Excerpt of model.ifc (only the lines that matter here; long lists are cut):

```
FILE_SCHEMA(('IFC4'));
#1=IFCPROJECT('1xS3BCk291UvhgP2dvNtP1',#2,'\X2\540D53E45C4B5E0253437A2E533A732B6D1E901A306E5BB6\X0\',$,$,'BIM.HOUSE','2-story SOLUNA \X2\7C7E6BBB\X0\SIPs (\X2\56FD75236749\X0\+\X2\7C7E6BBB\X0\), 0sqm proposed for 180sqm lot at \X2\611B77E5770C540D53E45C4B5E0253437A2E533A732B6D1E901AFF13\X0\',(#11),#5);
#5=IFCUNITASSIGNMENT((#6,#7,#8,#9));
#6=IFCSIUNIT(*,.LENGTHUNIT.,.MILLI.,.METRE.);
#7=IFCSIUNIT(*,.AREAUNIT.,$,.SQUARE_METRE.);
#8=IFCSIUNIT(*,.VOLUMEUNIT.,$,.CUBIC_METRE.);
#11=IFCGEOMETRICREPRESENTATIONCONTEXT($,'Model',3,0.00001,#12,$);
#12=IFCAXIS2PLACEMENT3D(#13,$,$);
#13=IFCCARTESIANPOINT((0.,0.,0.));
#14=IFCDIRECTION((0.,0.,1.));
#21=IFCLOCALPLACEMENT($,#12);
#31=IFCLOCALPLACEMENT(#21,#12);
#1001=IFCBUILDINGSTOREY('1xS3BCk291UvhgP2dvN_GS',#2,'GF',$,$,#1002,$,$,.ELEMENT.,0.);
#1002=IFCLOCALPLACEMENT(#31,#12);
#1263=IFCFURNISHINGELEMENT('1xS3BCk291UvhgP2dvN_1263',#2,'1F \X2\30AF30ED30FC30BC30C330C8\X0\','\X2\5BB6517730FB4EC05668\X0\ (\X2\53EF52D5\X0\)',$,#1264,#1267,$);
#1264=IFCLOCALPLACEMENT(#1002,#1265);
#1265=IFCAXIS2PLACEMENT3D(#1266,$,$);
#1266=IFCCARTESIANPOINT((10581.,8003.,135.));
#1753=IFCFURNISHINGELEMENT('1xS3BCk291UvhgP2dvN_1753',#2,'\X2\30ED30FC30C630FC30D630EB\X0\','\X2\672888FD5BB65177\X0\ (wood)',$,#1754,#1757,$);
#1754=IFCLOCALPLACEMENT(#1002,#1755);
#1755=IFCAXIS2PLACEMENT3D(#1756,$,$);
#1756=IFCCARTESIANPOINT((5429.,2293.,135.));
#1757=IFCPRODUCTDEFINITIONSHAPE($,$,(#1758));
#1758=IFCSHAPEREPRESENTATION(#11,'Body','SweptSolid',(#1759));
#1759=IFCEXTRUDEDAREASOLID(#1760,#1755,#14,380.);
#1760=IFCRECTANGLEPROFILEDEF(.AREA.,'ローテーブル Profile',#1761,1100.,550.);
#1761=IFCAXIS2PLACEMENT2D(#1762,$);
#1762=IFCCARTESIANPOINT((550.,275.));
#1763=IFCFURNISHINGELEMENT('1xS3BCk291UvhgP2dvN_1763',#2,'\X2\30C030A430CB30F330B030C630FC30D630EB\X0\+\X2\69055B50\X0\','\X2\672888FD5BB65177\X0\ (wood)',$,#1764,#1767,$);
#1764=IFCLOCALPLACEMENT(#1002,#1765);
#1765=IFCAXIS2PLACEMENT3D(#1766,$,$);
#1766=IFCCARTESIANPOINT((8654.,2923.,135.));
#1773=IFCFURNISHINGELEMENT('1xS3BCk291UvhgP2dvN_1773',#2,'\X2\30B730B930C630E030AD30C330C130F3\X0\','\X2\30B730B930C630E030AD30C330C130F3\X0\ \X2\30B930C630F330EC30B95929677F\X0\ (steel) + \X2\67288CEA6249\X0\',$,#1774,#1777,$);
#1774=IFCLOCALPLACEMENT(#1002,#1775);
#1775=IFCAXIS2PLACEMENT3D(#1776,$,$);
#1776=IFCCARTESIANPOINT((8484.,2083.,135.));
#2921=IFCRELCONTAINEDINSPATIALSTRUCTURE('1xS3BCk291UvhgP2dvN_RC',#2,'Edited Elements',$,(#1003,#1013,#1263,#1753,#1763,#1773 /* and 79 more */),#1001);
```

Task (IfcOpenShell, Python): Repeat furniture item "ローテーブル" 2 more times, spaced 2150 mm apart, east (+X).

```python
import numpy as np
import ifcopenshell
import ifcopenshell.api.geometry
import ifcopenshell.api.root
import ifcopenshell.util.element
import ifcopenshell.util.placement
import ifcopenshell.util.unit

model = ifcopenshell.open("model.ifc")
unit_scale = ifcopenshell.util.unit.calculate_unit_scale(model)


def reuse_history(source, copy):
    """copy_class also copies each property set's owner history, people and application; keep the originals."""
    for rel in copy.IsDefinedBy:
        if rel.is_a("IfcRelDefinesByProperties") and (history := rel.RelatingPropertyDefinition.OwnerHistory):
            rel.RelatingPropertyDefinition.OwnerHistory = source.OwnerHistory
            ifcopenshell.util.element.remove_deep2(model, history)


source = model.by_guid("1xS3BCk291UvhgP2dvN_1753")
base = ifcopenshell.util.placement.get_local_placement(source.ObjectPlacement)
step = np.array([1.0, 0.0, 0.0]) * 2.15 / unit_scale

for i in range(1, 3):
    copy = ifcopenshell.api.root.copy_class(model, product=source)
    copy.Representation = ifcopenshell.util.element.copy_deep(
        model, source.Representation, exclude=["IfcGeometricRepresentationContext", "IfcRepresentationMap"]
    )
    reuse_history(source, copy)
    matrix = base.copy()
    matrix[:3, 3] += i * step
    print("added at", matrix[:3, 3].round(3) + 0.0)
    ifcopenshell.api.geometry.edit_object_placement(model, product=copy, matrix=matrix, is_si=False)

model.write("model_updated.ifc")
```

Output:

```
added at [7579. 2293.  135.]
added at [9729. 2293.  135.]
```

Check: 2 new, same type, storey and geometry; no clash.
